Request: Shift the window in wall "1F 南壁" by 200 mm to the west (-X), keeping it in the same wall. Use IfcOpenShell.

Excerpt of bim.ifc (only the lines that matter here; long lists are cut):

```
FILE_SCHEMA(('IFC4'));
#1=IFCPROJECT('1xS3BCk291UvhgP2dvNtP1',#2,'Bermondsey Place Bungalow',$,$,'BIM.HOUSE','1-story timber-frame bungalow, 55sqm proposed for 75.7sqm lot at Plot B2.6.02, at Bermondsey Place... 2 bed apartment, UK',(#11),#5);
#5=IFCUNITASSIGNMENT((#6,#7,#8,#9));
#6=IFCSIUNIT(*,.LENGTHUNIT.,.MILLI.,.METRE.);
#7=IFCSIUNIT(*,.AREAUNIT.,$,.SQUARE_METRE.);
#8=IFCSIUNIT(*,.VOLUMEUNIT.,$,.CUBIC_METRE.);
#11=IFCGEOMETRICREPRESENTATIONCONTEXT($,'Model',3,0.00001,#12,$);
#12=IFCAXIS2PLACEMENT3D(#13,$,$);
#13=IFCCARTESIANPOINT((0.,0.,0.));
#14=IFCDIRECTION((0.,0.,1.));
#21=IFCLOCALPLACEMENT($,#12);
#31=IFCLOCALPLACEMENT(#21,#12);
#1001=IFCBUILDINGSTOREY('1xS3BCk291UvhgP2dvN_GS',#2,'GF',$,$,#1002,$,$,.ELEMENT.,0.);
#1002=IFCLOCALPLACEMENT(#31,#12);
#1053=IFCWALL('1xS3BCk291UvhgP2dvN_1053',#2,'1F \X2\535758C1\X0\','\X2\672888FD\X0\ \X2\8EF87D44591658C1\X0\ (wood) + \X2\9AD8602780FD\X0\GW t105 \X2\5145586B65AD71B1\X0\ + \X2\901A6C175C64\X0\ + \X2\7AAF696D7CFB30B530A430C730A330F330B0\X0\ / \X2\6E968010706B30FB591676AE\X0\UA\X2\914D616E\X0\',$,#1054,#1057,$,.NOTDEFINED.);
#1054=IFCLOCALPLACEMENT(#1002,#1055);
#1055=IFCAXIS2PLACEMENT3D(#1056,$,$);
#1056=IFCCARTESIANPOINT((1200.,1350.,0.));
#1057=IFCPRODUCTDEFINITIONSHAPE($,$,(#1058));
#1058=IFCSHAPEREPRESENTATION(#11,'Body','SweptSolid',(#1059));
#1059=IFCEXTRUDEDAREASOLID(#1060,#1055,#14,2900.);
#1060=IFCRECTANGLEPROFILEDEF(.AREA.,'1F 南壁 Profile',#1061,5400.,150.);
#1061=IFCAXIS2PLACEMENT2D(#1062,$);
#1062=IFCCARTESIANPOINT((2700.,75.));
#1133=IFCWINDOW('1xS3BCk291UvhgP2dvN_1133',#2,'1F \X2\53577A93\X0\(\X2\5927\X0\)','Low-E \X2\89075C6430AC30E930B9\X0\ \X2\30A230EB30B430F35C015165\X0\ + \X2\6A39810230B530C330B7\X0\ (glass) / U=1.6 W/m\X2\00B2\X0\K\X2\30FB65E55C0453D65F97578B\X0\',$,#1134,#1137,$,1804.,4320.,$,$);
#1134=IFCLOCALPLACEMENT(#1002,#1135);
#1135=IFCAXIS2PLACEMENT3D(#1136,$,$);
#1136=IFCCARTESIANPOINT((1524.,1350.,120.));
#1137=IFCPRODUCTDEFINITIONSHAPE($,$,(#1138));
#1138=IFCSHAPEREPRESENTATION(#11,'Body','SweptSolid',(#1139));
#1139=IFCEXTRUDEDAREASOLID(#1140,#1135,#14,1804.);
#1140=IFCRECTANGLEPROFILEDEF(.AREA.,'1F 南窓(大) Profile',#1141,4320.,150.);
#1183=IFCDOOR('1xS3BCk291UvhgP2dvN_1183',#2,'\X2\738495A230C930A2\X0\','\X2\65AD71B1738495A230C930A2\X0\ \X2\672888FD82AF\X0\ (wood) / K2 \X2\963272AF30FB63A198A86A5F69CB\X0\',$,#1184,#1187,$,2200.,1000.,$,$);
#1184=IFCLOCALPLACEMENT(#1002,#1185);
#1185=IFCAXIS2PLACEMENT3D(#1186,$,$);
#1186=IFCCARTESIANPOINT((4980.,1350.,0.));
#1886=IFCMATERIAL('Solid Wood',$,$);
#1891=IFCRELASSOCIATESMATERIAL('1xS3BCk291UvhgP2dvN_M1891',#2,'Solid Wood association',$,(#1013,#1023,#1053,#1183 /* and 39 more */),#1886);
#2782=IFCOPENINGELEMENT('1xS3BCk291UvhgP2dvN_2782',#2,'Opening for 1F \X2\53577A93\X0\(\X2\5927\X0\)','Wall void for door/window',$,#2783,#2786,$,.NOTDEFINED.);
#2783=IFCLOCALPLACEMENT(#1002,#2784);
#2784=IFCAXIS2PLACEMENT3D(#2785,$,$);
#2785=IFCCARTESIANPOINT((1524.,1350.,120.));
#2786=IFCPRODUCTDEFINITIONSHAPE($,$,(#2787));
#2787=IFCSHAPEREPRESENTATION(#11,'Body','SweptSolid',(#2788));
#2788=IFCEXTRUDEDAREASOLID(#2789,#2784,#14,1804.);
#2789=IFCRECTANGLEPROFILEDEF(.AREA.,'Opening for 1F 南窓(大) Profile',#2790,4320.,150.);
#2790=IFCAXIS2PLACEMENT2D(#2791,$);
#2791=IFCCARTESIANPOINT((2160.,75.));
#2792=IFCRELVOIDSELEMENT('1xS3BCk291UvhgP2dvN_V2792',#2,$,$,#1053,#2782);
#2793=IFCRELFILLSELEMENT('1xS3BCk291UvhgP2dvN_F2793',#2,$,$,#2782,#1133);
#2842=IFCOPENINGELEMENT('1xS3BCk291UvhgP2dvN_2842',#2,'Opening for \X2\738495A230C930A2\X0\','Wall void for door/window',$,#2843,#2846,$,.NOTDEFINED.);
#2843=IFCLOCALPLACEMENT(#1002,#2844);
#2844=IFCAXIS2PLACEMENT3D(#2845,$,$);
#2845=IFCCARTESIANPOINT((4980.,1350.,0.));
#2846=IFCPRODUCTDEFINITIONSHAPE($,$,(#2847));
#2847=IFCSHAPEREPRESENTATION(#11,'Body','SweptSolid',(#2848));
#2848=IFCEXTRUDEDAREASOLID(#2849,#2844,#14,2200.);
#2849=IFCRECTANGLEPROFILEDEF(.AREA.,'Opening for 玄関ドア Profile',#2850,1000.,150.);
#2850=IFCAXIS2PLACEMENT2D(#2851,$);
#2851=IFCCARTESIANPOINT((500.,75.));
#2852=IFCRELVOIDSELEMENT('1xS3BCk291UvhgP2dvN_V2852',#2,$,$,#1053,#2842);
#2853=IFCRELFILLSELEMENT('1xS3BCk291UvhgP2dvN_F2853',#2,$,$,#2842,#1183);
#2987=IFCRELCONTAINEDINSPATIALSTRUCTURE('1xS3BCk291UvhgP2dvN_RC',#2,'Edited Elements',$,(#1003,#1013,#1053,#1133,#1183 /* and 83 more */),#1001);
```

```python
import ifcopenshell
import ifcopenshell.api.geometry
import ifcopenshell.util.placement
import ifcopenshell.util.unit

model = ifcopenshell.open("bim.ifc")
unit_scale = ifcopenshell.util.unit.calculate_unit_scale(model)

window = model.by_guid("1xS3BCk291UvhgP2dvN_1133")
opening = window.FillsVoids[0].RelatingOpeningElement
wall = opening.VoidsElements[0].RelatingBuildingElement

wall_matrix = ifcopenshell.util.placement.get_local_placement(wall.ObjectPlacement)
shift = wall_matrix[:3, 0] * -0.2 / unit_scale
before = ifcopenshell.util.placement.get_local_placement(window.ObjectPlacement)[:3, 3].copy()

# The window is not placed relative to its opening, so move both.
for product in (opening, window):
    matrix = ifcopenshell.util.placement.get_local_placement(product.ObjectPlacement)
    matrix[:3, 3] += shift
    ifcopenshell.api.geometry.edit_object_placement(model, product=product, matrix=matrix, is_si=False)

after = ifcopenshell.util.placement.get_local_placement(window.ObjectPlacement)[:3, 3]
print("window moved by", (after - before).round(3) + 0.0)

model.write("bim_v2.ifc")
```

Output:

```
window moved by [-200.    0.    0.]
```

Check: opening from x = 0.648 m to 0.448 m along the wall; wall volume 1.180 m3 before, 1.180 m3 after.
